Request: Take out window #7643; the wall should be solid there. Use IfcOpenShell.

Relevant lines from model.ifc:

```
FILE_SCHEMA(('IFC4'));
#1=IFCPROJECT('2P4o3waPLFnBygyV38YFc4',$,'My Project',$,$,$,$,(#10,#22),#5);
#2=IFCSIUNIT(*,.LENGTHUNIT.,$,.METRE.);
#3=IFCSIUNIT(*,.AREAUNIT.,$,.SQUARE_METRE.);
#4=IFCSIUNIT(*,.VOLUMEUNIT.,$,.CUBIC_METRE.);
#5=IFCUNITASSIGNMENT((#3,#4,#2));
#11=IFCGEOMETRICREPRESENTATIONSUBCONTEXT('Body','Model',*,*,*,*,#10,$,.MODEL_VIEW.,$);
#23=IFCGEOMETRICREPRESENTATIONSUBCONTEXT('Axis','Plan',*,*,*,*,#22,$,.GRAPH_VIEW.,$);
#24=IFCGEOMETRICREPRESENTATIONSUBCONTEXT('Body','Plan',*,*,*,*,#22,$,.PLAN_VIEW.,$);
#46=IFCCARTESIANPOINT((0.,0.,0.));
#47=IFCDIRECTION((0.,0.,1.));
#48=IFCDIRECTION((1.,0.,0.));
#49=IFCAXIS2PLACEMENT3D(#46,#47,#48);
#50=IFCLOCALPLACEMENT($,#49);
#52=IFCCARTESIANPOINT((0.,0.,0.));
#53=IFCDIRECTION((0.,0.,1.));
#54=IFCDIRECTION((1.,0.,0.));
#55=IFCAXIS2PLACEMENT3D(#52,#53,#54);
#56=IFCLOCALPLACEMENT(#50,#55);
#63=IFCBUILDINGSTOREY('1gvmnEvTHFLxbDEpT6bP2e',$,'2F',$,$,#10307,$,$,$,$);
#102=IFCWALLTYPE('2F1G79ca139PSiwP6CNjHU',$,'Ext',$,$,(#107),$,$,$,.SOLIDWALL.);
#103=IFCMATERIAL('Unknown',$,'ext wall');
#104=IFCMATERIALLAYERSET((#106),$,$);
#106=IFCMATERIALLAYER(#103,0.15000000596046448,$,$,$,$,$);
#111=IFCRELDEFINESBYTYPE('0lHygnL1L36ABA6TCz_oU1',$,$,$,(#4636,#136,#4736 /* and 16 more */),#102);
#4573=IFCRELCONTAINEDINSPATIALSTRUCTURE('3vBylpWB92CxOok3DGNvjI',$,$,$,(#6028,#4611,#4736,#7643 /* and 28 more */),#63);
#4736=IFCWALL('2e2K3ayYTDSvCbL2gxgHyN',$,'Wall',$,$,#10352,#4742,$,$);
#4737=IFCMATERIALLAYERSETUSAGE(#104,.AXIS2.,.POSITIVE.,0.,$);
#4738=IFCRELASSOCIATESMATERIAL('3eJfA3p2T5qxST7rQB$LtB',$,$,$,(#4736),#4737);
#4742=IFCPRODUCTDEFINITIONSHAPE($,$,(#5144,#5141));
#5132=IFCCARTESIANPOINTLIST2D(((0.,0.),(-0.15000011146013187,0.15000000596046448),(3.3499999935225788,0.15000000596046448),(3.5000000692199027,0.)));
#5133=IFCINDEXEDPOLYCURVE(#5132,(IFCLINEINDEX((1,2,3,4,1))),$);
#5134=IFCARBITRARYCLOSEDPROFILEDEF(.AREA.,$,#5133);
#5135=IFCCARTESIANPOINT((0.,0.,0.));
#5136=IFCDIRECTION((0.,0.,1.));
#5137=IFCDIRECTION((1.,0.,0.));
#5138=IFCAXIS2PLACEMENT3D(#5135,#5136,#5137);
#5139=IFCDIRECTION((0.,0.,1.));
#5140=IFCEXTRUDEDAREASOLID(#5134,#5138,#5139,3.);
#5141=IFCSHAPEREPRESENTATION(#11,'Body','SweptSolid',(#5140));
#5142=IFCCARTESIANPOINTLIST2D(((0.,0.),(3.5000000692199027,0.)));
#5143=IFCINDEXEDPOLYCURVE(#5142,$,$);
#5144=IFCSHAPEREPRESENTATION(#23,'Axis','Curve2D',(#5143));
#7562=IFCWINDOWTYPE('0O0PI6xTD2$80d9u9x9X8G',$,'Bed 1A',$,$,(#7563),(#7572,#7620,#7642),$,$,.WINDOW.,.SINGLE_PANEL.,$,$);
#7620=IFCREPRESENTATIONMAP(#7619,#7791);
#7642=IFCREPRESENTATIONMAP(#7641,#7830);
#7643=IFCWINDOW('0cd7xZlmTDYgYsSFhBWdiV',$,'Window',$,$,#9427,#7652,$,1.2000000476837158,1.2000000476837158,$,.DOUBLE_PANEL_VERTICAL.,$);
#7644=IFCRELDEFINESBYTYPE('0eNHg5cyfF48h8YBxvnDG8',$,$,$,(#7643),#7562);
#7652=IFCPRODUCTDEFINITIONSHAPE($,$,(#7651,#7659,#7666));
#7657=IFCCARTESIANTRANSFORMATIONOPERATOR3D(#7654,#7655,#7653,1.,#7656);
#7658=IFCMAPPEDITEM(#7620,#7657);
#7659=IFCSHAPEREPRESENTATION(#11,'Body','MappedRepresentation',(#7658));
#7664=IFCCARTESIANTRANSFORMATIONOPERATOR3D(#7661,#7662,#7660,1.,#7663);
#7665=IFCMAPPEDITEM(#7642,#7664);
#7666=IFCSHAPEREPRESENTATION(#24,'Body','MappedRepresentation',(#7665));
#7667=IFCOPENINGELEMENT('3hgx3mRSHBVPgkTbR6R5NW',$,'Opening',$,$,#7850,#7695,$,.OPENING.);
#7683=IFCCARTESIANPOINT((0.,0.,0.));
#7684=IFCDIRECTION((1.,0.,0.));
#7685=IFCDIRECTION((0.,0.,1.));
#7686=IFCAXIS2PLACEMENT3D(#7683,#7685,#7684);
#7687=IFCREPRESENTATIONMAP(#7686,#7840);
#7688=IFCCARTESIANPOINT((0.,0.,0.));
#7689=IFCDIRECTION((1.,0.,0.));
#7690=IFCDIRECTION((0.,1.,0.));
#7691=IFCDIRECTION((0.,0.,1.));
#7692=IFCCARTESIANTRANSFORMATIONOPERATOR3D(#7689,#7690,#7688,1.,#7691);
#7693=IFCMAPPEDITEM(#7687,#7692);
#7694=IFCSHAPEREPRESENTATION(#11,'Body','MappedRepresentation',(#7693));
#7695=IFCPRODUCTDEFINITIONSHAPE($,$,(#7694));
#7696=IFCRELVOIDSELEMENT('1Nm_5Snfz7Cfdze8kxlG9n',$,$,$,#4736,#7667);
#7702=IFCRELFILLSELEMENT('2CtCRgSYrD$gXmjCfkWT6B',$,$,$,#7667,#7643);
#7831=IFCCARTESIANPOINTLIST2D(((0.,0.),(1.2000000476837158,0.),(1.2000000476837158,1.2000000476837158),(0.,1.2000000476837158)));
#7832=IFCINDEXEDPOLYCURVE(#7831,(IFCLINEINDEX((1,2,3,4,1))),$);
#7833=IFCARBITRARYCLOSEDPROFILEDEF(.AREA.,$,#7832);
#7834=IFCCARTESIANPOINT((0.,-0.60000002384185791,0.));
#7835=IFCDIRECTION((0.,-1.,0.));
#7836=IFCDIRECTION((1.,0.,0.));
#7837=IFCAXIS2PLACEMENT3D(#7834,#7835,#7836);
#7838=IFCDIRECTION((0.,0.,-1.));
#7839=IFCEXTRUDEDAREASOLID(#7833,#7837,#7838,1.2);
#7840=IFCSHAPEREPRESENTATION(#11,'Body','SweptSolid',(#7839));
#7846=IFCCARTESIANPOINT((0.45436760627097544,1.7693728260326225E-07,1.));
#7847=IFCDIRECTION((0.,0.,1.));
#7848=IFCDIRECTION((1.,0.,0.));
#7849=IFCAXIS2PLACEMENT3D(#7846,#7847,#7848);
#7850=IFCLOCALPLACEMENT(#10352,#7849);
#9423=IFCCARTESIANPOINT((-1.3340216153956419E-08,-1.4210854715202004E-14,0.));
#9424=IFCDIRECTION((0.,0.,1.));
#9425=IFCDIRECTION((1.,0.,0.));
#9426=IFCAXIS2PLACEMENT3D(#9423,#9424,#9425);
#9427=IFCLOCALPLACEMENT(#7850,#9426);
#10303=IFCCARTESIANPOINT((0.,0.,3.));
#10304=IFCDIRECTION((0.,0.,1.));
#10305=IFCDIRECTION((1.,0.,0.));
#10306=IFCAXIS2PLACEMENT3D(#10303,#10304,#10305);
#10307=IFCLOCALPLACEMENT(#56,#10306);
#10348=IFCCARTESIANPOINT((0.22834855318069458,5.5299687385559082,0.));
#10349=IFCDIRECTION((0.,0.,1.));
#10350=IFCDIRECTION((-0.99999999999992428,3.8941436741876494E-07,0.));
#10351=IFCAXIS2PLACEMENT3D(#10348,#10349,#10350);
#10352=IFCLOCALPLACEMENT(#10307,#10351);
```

```python
import ifcopenshell
import ifcopenshell.api.feature
import ifcopenshell.api.root
import ifcopenshell.geom
import ifcopenshell.util.shape

model = ifcopenshell.open("model.ifc")
settings = ifcopenshell.geom.settings()


def volume(element):
    """Net volume in cubic metres, openings subtracted."""
    shape = ifcopenshell.geom.create_shape(settings, element)
    return ifcopenshell.util.shape.get_volume(shape.geometry)


window = model.by_guid("0cd7xZlmTDYgYsSFhBWdiV")
opening = window.FillsVoids[0].RelatingOpeningElement
wall = opening.VoidsElements[0].RelatingBuildingElement
before = volume(wall)

ifcopenshell.api.root.remove_product(model, product=window)
ifcopenshell.api.feature.remove_feature(model, feature=opening)

after = volume(wall)

print(f"wall volume {before:.3f} -> {after:.3f} m3")

model.write("model-out.ifc")
```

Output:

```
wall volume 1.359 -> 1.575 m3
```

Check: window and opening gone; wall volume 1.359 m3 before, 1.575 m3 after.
